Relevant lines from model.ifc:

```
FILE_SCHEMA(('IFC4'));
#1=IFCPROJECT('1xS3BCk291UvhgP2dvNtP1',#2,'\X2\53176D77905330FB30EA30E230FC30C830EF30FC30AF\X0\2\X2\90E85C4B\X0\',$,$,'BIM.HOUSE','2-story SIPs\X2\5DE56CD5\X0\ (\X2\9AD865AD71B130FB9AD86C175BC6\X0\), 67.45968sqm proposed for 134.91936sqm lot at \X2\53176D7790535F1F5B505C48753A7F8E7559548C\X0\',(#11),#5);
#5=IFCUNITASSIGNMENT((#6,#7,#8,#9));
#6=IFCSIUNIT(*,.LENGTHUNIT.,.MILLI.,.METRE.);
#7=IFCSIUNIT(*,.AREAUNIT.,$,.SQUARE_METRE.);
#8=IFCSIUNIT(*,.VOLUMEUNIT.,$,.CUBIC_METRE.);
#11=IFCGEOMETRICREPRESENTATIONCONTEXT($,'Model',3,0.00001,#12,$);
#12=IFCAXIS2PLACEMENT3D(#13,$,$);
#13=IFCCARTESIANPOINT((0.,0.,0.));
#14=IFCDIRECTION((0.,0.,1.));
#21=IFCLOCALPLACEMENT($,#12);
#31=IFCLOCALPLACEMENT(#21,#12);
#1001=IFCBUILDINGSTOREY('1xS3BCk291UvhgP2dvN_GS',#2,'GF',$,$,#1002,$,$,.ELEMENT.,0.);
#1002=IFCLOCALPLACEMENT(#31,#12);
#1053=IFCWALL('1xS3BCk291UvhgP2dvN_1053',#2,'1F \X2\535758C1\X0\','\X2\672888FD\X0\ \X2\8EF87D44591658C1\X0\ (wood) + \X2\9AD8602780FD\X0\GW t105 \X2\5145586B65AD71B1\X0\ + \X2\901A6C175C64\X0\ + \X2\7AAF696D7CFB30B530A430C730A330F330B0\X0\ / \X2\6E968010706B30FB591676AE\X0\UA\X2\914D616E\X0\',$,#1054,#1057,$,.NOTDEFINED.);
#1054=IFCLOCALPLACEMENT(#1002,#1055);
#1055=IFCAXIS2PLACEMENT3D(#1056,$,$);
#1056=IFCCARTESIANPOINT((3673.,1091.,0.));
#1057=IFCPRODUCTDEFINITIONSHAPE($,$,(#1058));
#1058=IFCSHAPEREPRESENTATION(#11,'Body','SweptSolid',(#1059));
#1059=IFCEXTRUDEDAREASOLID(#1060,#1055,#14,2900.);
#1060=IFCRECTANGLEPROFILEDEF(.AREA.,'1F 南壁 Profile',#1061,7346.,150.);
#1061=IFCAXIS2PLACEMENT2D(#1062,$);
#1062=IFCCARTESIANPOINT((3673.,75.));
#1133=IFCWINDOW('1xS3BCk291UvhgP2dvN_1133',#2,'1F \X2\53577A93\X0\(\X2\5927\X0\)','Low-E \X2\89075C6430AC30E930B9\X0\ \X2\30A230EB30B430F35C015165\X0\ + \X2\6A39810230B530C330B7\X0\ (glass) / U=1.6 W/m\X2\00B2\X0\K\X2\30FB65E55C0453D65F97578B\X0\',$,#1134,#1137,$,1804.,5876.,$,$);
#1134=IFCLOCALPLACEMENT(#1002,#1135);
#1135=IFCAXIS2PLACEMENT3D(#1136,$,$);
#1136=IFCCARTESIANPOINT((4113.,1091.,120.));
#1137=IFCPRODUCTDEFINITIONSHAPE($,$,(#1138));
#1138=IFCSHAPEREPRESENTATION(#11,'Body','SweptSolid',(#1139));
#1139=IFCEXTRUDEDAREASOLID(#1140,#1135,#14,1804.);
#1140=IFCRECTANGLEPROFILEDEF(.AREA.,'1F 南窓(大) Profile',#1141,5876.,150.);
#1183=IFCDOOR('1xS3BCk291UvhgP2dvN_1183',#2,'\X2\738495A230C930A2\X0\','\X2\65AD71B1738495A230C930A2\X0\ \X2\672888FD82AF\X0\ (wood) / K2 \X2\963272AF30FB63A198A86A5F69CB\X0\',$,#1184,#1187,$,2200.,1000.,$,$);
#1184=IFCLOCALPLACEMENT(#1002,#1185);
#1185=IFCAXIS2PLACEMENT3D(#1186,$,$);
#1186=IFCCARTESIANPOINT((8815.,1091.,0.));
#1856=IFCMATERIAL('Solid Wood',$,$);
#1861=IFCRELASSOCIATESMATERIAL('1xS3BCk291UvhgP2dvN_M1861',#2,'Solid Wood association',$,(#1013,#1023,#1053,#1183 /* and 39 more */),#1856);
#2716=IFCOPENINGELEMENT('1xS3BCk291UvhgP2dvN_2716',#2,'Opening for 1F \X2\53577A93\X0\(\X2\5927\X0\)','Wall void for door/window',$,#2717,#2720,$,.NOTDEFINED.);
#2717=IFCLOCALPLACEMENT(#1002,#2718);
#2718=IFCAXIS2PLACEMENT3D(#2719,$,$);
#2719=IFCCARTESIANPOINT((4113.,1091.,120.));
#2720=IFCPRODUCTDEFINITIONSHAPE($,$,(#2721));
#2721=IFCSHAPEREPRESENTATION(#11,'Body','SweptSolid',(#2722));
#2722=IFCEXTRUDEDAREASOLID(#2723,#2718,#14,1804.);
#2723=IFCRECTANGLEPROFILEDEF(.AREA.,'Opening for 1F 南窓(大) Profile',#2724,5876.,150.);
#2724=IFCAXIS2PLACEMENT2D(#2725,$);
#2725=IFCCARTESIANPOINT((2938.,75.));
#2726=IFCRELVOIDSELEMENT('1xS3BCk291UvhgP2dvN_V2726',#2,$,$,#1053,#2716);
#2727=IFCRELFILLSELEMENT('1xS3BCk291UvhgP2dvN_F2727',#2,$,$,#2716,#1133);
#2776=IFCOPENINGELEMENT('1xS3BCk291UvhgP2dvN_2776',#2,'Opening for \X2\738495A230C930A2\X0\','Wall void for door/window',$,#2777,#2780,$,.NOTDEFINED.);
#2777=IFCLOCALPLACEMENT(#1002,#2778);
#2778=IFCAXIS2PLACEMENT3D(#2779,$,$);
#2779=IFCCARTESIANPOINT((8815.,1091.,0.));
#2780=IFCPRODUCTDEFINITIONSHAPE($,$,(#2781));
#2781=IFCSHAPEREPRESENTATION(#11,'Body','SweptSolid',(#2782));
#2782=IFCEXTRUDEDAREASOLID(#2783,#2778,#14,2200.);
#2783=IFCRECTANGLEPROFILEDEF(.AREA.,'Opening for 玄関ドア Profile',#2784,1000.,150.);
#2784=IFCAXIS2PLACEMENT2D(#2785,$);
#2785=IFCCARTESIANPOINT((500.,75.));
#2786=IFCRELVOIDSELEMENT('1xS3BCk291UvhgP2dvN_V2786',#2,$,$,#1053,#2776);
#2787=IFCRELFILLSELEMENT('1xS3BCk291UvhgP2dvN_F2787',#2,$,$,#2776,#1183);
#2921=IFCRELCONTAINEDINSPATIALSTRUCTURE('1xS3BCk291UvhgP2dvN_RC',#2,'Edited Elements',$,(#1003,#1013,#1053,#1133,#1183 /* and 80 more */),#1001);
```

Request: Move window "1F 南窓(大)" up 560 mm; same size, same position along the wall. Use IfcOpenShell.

```python
import numpy as np
import ifcopenshell
import ifcopenshell.api.geometry
import ifcopenshell.util.placement
import ifcopenshell.util.unit

model = ifcopenshell.open("model.ifc")
unit_scale = ifcopenshell.util.unit.calculate_unit_scale(model)

window = model.by_guid("1xS3BCk291UvhgP2dvN_1133")
opening = window.FillsVoids[0].RelatingOpeningElement
dz = 0.56 / unit_scale

shift = np.array([0.0, 0.0, dz])
# The window is not placed relative to its opening, so move both.
for product in (opening, window):
    matrix = ifcopenshell.util.placement.get_local_placement(product.ObjectPlacement)
    matrix[:3, 3] += shift
    ifcopenshell.api.geometry.edit_object_placement(model, product=product, matrix=matrix, is_si=False)

print(f"moved by {dz * unit_scale:+.3f} m")

model.write("model_edited.ifc")
```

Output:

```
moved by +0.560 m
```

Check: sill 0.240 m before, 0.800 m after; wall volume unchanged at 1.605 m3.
